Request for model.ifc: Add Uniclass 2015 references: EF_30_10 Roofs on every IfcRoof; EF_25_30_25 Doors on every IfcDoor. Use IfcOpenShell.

First a look at what the model holds.

```python
import ifcopenshell

model = ifcopenshell.open("model.ifc")
print(model.schema)
print("classifications:", [c.Name for c in model.by_type("IfcClassification")])
for ifc_class in ("IfcDoor", "IfcRoof", "IfcStair", "IfcWall", "IfcWindow"):
    print(ifc_class, len(model.by_type(ifc_class)))
```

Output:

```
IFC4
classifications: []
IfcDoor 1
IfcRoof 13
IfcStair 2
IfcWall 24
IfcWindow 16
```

```python
import ifcopenshell
import ifcopenshell.api.classification

model = ifcopenshell.open("model.ifc")

system = ifcopenshell.api.classification.add_classification(model, classification="Uniclass 2015")

codes = {
    "IfcRoof": ("EF_30_10", "Roofs"),
    "IfcDoor": ("EF_25_30_25", "Doors"),
}
for ifc_class, (code, name) in codes.items():
    products = model.by_type(ifc_class)
    ifcopenshell.api.classification.add_reference(
        model, products=products, classification=system, identification=code, name=name
    )
    print(code, len(products))

model.write("model-out.ifc")
```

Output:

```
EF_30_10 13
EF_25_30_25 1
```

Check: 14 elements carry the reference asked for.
